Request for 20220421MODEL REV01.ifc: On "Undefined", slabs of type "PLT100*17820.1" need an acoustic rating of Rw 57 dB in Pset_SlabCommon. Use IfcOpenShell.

First a look at what the model holds.

```python
import ifcopenshell
import ifcopenshell.util.element

model = ifcopenshell.open("20220421MODEL REV01.ifc")
print(model.schema)
storey = next(s for s in model.by_type("IfcBuildingStorey") if s.Name == "Undefined")
slabs = [e for e in ifcopenshell.util.element.get_decomposition(storey) if e.is_a("IfcSlab")]
seen = {}
for e in slabs:
    element_type = ifcopenshell.util.element.get_type(e)
    key = (element_type.Name if element_type != e and element_type else None, ifcopenshell.util.element.get_pset(e, "Pset_SlabCommon", "AcousticRating"))
    seen[key] = seen.get(key, 0) + 1
for (name, value), count in sorted(seen.items(), key=str):
    print(count, "x", name, "|", value)
```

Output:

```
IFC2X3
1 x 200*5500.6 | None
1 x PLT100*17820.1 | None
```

```python
import ifcopenshell
import ifcopenshell.api.pset
import ifcopenshell.util.element

model = ifcopenshell.open("20220421MODEL REV01.ifc")

storey = next(s for s in model.by_type("IfcBuildingStorey") if s.Name == "Undefined")
slabs = [e for e in ifcopenshell.util.element.get_decomposition(storey) if e.is_a("IfcSlab")]

count = 0
for e in slabs:
    element_type = ifcopenshell.util.element.get_type(e)
    if element_type in (None, e) or element_type.Name != "PLT100*17820.1":
        continue
    # add_pset returns the element's existing set when there is one.
    pset = ifcopenshell.api.pset.add_pset(model, product=e, name="Pset_SlabCommon")
    ifcopenshell.api.pset.edit_pset(model, pset=pset, properties={"AcousticRating": "Rw 57 dB"})
    count += 1

print(count, "slabs updated")

model.write("20220421MODEL REV01_updated.ifc")
```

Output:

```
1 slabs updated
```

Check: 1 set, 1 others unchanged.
